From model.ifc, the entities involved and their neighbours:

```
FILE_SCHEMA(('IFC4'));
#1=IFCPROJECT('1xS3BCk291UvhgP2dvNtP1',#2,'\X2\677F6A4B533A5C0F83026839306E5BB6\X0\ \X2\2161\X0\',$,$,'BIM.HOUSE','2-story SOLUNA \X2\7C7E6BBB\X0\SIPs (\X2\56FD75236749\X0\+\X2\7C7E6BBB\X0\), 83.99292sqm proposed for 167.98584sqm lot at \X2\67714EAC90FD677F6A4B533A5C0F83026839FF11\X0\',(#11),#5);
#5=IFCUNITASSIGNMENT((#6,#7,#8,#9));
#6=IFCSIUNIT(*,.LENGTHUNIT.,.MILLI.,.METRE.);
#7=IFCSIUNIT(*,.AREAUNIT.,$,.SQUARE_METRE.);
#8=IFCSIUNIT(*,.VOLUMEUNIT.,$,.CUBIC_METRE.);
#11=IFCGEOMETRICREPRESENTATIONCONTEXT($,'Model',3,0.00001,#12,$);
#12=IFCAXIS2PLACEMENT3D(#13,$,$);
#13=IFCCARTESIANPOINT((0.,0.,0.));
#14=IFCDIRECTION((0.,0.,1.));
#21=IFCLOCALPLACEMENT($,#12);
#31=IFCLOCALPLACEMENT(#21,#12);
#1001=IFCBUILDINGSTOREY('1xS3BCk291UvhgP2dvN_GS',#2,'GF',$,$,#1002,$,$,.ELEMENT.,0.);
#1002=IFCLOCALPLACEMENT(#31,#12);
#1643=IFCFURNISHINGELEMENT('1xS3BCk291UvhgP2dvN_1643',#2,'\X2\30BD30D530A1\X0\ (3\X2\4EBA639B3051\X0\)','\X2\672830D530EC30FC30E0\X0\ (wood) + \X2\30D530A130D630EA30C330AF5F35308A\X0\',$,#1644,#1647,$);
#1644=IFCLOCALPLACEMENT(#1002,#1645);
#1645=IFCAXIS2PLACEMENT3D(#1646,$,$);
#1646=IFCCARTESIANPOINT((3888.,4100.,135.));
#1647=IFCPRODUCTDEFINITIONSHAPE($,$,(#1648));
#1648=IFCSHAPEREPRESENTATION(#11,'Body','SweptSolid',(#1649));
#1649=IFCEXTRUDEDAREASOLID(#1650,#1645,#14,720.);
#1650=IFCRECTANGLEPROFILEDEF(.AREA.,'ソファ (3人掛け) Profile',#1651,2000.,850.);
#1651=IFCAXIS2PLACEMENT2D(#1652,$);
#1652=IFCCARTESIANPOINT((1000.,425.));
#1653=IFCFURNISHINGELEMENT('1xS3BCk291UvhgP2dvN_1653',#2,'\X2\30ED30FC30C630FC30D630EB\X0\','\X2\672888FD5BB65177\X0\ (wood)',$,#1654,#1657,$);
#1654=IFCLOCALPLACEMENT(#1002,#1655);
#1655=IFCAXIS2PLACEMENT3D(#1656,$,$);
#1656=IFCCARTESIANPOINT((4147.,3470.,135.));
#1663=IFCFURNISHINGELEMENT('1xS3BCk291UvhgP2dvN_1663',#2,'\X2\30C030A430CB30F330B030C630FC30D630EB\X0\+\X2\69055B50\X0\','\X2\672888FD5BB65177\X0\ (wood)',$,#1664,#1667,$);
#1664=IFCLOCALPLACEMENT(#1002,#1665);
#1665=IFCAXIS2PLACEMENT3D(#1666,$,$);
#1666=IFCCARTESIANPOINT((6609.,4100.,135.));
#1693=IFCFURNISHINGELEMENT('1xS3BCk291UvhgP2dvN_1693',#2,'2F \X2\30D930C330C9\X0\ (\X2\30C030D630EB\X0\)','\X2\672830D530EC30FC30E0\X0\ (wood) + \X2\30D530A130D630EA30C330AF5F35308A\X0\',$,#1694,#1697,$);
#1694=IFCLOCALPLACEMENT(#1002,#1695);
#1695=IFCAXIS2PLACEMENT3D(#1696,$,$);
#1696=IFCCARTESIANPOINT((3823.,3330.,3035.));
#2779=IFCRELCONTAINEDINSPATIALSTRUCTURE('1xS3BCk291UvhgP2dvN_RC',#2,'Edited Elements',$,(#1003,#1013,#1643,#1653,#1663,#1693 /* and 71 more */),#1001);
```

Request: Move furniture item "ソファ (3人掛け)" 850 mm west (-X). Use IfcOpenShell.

```python
import ifcopenshell
import ifcopenshell.api.geometry
import ifcopenshell.util.placement
import ifcopenshell.util.unit

model = ifcopenshell.open("model.ifc")
unit_scale = ifcopenshell.util.unit.calculate_unit_scale(model)

item = model.by_guid("1xS3BCk291UvhgP2dvN_1643")
matrix = ifcopenshell.util.placement.get_local_placement(item.ObjectPlacement)
matrix[0, 3] -= 0.85 / unit_scale
ifcopenshell.api.geometry.edit_object_placement(model, product=item, matrix=matrix, is_si=False)

print(ifcopenshell.util.placement.get_local_placement(item.ObjectPlacement).round(3) + 0.0)

model.write("model_rev.ifc")
```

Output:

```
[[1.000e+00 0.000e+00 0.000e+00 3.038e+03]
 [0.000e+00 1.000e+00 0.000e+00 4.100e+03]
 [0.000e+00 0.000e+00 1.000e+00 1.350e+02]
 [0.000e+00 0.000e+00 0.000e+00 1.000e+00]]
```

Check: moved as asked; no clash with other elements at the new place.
